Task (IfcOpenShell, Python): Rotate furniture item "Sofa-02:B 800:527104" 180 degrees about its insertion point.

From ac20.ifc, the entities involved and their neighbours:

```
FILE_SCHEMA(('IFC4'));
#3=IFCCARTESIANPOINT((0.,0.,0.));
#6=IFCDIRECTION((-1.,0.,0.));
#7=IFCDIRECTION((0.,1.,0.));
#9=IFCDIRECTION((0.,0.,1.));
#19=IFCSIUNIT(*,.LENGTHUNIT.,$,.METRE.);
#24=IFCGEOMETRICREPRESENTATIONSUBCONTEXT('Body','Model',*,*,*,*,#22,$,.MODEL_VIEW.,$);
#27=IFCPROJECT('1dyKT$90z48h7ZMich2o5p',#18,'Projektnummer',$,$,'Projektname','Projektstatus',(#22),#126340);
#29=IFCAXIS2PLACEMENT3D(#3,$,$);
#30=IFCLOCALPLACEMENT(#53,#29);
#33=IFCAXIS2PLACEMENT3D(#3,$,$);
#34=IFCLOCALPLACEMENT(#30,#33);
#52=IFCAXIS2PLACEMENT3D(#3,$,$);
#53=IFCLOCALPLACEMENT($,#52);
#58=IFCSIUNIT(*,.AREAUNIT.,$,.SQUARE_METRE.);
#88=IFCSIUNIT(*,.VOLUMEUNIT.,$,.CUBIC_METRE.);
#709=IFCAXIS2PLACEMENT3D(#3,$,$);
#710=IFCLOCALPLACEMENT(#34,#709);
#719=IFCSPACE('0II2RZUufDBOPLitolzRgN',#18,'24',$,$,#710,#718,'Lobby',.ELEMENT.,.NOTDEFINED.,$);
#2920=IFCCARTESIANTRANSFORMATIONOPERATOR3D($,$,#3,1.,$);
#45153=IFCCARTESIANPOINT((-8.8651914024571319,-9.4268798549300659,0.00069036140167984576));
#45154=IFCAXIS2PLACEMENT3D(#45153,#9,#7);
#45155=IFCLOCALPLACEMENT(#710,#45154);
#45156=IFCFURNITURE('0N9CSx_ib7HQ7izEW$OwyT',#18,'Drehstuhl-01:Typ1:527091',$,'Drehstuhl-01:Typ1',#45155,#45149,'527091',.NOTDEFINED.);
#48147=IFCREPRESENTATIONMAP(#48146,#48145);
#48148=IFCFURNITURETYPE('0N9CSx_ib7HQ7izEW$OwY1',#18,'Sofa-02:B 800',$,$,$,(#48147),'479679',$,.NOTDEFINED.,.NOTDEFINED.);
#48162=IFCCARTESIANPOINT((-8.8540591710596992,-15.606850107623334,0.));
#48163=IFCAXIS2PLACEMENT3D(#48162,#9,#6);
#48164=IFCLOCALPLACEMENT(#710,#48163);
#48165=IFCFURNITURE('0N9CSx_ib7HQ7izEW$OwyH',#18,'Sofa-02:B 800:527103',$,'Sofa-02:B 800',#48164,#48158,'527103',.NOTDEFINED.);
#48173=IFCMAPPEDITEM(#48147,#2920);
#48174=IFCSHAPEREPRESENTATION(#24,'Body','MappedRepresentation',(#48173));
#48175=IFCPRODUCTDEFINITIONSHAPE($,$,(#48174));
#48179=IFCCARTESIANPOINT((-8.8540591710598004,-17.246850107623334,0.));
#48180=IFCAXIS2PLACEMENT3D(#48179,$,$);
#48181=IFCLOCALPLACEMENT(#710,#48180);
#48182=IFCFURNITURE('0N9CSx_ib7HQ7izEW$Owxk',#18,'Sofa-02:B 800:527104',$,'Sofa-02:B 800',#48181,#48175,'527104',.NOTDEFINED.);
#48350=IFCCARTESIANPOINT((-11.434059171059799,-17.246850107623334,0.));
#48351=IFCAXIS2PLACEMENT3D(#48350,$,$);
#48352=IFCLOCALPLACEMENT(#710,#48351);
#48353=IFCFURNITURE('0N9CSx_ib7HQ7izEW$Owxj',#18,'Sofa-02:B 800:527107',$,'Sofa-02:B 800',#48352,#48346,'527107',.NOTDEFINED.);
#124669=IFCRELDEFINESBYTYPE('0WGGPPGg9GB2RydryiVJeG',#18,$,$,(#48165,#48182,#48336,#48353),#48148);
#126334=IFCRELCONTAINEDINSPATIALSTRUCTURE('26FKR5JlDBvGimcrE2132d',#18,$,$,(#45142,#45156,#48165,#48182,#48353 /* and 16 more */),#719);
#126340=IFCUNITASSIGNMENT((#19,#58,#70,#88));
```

```python
import ifcopenshell
import ifcopenshell.api.geometry
import ifcopenshell.util.placement

model = ifcopenshell.open("ac20.ifc")

item = model.by_guid("0N9CSx_ib7HQ7izEW$Owxk")
matrix = ifcopenshell.util.placement.get_local_placement(item.ObjectPlacement)
matrix = matrix @ ifcopenshell.util.placement.rotation(180, "Z")
ifcopenshell.api.geometry.edit_object_placement(model, product=item, matrix=matrix, is_si=False)

print(ifcopenshell.util.placement.get_local_placement(item.ObjectPlacement).round(3) + 0.0)

model.write("ac20_edited.ifc")
```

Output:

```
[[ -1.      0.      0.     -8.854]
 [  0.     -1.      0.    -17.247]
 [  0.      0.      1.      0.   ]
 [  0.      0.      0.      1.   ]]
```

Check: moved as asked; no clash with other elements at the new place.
